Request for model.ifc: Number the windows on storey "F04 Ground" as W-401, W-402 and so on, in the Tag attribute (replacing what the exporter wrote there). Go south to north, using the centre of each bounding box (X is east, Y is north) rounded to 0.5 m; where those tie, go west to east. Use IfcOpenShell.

First a look at what the model holds.

```python
import ifcopenshell
import ifcopenshell.util.element
import ifcopenshell.util.placement

model = ifcopenshell.open("model.ifc")
print(model.schema)
storey = next(s for s in model.by_type("IfcBuildingStorey") if s.Name == "F04 Ground")
windows = [e for e in ifcopenshell.util.element.get_decomposition(storey) if e.is_a("IfcWindow")]
for e in sorted(windows, key=lambda e: e.id()):
    origin = ifcopenshell.util.placement.get_local_placement(e.ObjectPlacement)[:3, 3]
    print(e.id(), e.Tag, e.Name, origin.round(2) + 0.0, sep=" | ")
```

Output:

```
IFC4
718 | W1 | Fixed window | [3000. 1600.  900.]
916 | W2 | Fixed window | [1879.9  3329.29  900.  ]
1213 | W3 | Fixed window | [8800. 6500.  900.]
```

```python
import ifcopenshell
import ifcopenshell.geom
import ifcopenshell.util.element
import ifcopenshell.util.shape

model = ifcopenshell.open("model.ifc")
settings = ifcopenshell.geom.settings()
settings.set("use-world-coords", True)


def centre(element):
    shape = ifcopenshell.geom.create_shape(settings, element)
    return ifcopenshell.util.shape.get_bbox_centroid(shape.geometry)


storey = next(s for s in model.by_type("IfcBuildingStorey") if s.Name == "F04 Ground")
windows = [e for e in ifcopenshell.util.element.get_decomposition(storey) if e.is_a("IfcWindow")]

# Insertion points can sit at a corner or the storey origin, so sort by the geometry (in metres).
centres = {e: centre(e) for e in windows}
windows.sort(key=lambda e: (round(centres[e][1] / 0.5), centres[e][0]))

for i, e in enumerate(windows, start=1):
    number = f"W-4{i:02d}"
    e.Tag = number
    print(e.id(), number)

model.write("model_updated.ifc")
```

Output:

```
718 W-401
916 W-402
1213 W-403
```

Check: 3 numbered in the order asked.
